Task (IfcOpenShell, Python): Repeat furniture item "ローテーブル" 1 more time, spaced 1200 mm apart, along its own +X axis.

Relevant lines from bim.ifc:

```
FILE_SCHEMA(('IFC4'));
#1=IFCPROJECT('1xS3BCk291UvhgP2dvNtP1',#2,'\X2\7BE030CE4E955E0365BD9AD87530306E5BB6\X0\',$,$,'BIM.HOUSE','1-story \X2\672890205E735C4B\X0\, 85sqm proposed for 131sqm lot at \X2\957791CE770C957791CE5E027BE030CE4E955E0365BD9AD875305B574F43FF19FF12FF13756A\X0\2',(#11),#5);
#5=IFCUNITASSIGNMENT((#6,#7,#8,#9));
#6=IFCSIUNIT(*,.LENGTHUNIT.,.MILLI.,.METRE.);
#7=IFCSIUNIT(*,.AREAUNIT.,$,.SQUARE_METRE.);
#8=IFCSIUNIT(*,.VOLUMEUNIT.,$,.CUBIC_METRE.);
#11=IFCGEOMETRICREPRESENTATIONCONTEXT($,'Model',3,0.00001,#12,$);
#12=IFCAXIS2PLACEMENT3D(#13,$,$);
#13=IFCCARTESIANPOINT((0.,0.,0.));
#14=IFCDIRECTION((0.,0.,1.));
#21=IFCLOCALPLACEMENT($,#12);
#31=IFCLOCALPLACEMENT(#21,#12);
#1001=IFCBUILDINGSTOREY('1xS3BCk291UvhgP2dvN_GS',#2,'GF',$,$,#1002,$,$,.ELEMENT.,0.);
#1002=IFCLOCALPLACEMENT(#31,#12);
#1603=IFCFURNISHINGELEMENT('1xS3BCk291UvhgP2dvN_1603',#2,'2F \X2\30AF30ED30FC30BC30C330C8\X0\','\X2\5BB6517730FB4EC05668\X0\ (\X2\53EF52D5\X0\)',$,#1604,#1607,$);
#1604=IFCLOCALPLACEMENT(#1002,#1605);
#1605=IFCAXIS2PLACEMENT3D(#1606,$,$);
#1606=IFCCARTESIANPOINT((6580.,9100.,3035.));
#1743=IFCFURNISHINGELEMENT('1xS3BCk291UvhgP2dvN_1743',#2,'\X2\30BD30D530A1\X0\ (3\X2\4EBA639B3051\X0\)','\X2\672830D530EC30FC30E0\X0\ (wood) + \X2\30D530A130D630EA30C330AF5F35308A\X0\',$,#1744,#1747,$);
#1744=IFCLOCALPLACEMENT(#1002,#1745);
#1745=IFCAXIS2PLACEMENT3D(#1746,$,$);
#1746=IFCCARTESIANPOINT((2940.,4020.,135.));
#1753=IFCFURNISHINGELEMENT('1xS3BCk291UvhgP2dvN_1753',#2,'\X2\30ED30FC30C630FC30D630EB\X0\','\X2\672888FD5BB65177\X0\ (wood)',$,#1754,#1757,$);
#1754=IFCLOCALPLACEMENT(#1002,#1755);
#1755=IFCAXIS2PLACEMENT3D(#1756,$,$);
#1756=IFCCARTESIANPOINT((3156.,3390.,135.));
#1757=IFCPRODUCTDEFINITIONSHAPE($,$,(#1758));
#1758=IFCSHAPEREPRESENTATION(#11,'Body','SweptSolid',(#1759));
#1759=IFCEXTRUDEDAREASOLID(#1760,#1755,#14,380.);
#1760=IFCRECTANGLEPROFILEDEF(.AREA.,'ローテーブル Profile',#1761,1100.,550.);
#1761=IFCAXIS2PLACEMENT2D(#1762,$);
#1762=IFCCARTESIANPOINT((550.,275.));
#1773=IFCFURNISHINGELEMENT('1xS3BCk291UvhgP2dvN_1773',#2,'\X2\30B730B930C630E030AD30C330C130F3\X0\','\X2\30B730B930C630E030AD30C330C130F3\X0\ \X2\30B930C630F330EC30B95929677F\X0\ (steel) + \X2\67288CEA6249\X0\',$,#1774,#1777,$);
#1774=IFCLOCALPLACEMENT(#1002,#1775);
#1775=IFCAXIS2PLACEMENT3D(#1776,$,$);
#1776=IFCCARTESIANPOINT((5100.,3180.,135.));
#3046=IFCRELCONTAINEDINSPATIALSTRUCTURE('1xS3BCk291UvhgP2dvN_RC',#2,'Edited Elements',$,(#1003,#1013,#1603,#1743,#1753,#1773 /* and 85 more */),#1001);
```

```python
import ifcopenshell
import ifcopenshell.api.geometry
import ifcopenshell.api.root
import ifcopenshell.util.element
import ifcopenshell.util.placement

model = ifcopenshell.open("bim.ifc")


def reuse_history(source, copy):
    """copy_class also copies each property set's owner history, people and application; keep the originals."""
    for rel in copy.IsDefinedBy:
        if rel.is_a("IfcRelDefinesByProperties") and (history := rel.RelatingPropertyDefinition.OwnerHistory):
            rel.RelatingPropertyDefinition.OwnerHistory = source.OwnerHistory
            ifcopenshell.util.element.remove_deep2(model, history)


source = model.by_guid("1xS3BCk291UvhgP2dvN_1753")
base = ifcopenshell.util.placement.get_local_placement(source.ObjectPlacement)
step = base[:3, 0] * 1200.0

for i in range(1, 2):
    copy = ifcopenshell.api.root.copy_class(model, product=source)
    copy.Representation = ifcopenshell.util.element.copy_deep(
        model, source.Representation, exclude=["IfcGeometricRepresentationContext", "IfcRepresentationMap"]
    )
    reuse_history(source, copy)
    matrix = base.copy()
    matrix[:3, 3] += i * step
    print("added at", matrix[:3, 3].round(3) + 0.0)
    ifcopenshell.api.geometry.edit_object_placement(model, product=copy, matrix=matrix, is_si=False)

model.write("bim_updated.ifc")
```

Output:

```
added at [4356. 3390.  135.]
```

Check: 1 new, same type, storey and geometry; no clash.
